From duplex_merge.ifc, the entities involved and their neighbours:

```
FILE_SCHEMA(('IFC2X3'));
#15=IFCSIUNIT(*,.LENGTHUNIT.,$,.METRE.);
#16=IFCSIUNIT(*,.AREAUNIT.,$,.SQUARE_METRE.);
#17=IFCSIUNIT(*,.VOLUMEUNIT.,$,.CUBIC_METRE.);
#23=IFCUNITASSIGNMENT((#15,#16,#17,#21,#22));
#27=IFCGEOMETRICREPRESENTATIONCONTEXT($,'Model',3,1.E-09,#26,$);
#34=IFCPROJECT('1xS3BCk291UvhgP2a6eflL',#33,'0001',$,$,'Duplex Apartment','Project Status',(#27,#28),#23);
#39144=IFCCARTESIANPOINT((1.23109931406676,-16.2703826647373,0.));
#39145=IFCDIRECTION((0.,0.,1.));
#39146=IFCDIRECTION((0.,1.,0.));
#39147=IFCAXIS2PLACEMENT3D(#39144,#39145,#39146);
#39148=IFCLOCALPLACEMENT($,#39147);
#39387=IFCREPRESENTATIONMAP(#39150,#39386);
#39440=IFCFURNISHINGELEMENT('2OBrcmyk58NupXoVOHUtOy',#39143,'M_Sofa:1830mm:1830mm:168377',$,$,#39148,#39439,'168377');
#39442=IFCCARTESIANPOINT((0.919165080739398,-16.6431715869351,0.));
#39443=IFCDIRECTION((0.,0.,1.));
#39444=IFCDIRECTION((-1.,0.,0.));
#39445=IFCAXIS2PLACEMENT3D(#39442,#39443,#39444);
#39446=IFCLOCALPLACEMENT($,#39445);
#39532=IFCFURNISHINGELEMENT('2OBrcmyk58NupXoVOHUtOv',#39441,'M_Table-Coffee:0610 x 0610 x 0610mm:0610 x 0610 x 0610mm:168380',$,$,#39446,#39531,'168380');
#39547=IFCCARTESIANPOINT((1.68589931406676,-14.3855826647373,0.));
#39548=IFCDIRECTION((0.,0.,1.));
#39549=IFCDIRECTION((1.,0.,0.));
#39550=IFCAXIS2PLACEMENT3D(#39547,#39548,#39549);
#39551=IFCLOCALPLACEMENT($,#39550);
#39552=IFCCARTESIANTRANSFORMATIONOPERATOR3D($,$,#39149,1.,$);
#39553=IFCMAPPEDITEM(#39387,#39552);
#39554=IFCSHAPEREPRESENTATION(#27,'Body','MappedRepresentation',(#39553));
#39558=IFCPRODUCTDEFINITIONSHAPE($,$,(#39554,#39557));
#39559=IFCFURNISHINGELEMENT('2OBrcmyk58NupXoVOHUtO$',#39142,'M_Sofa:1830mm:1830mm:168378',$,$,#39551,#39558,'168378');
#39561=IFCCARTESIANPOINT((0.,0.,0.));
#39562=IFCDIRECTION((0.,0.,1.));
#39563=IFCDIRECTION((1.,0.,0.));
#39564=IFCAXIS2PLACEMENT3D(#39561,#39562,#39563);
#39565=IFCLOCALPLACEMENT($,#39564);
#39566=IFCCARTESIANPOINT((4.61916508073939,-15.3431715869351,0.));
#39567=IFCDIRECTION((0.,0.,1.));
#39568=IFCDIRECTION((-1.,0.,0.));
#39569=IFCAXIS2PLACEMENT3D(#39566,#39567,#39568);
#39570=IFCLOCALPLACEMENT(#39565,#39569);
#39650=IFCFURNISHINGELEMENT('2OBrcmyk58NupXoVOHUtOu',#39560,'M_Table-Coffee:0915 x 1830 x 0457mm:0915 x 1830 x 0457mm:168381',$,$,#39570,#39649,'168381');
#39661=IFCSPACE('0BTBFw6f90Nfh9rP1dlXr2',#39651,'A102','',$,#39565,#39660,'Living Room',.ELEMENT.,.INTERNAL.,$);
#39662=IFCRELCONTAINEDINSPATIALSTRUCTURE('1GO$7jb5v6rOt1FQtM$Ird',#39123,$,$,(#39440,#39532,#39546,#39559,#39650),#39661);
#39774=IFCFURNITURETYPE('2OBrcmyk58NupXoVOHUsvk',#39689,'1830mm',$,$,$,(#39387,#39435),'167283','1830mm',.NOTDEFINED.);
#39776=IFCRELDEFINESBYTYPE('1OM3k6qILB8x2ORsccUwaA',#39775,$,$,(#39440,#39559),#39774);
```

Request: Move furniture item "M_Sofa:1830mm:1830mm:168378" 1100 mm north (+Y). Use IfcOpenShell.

```python
import ifcopenshell
import ifcopenshell.api.geometry
import ifcopenshell.util.placement

model = ifcopenshell.open("duplex_merge.ifc")

item = model.by_guid("2OBrcmyk58NupXoVOHUtO$")
matrix = ifcopenshell.util.placement.get_local_placement(item.ObjectPlacement)
matrix[1, 3] += 1.1
ifcopenshell.api.geometry.edit_object_placement(model, product=item, matrix=matrix, is_si=False)

print(ifcopenshell.util.placement.get_local_placement(item.ObjectPlacement).round(3) + 0.0)

model.write("duplex_merge_edited.ifc")
```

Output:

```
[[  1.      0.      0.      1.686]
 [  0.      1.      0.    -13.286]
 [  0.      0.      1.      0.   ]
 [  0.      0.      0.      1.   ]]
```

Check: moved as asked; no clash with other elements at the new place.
